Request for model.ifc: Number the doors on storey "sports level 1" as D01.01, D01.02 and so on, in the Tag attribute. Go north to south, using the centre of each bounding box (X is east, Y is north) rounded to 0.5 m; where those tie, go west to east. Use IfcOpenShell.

First a look at what the model holds.

```python
import ifcopenshell
import ifcopenshell.util.element
import ifcopenshell.util.placement

model = ifcopenshell.open("model.ifc")
print(model.schema)
storey = next(s for s in model.by_type("IfcBuildingStorey") if s.Name == "sports level 1")
doors = [e for e in ifcopenshell.util.element.get_decomposition(storey) if e.is_a("IfcDoor")]
for e in sorted(doors, key=lambda e: e.id()):
    origin = ifcopenshell.util.placement.get_local_placement(e.ObjectPlacement)[:3, 3]
    print(e.id(), e.Tag, e.Name, origin.round(2) + 0.0, sep=" | ")
```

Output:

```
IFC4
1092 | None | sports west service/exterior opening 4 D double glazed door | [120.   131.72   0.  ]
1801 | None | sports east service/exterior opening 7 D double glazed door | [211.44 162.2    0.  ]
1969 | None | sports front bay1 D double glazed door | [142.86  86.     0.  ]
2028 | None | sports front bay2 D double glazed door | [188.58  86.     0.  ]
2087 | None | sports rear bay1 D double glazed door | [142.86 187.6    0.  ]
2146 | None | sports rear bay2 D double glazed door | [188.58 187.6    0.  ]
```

```python
import ifcopenshell
import ifcopenshell.geom
import ifcopenshell.util.element
import ifcopenshell.util.shape

model = ifcopenshell.open("model.ifc")
settings = ifcopenshell.geom.settings()
settings.set("use-world-coords", True)


def centre(element):
    shape = ifcopenshell.geom.create_shape(settings, element)
    return ifcopenshell.util.shape.get_bbox_centroid(shape.geometry)


storey = next(s for s in model.by_type("IfcBuildingStorey") if s.Name == "sports level 1")
doors = [e for e in ifcopenshell.util.element.get_decomposition(storey) if e.is_a("IfcDoor")]

# Insertion points can sit at a corner or the storey origin, so sort by the geometry (in metres).
centres = {e: centre(e) for e in doors}
doors.sort(key=lambda e: (-round(centres[e][1] / 0.5), centres[e][0]))

for i, e in enumerate(doors, start=1):
    number = f"D01.{i:02d}"
    e.Tag = number
    print(e.id(), number)

model.write("model_updated.ifc")
```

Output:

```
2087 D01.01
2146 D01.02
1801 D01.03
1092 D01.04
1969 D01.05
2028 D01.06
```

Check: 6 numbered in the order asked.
